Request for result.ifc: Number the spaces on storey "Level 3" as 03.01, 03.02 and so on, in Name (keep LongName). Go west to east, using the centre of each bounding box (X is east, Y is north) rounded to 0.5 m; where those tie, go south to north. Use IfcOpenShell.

First a look at what the model holds.

```python
import ifcopenshell
import ifcopenshell.util.element
import ifcopenshell.util.placement

model = ifcopenshell.open("result.ifc")
print(model.schema)
storey = next(s for s in model.by_type("IfcBuildingStorey") if s.Name == "Level 3")
spaces = [e for e in ifcopenshell.util.element.get_decomposition(storey) if e.is_a("IfcSpace")]
for e in sorted(spaces, key=lambda e: e.id()):
    origin = ifcopenshell.util.placement.get_local_placement(e.ObjectPlacement)[:3, 3]
    print(e.id(), e.Name, e.LongName, origin.round(2) + 0.0, sep=" | ")
```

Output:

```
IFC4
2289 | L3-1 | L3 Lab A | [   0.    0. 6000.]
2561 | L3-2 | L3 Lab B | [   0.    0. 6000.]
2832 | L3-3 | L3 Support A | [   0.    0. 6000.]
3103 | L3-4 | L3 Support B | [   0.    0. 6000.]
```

```python
import ifcopenshell
import ifcopenshell.geom
import ifcopenshell.util.element
import ifcopenshell.util.shape

model = ifcopenshell.open("result.ifc")
settings = ifcopenshell.geom.settings()
settings.set("use-world-coords", True)


def centre(element):
    shape = ifcopenshell.geom.create_shape(settings, element)
    return ifcopenshell.util.shape.get_bbox_centroid(shape.geometry)


storey = next(s for s in model.by_type("IfcBuildingStorey") if s.Name == "Level 3")
spaces = [e for e in ifcopenshell.util.element.get_decomposition(storey) if e.is_a("IfcSpace")]

# Insertion points can sit at a corner or the storey origin, so sort by the geometry (in metres).
centres = {e: centre(e) for e in spaces}
spaces.sort(key=lambda e: (round(centres[e][0] / 0.5), centres[e][1]))

for i, e in enumerate(spaces, start=1):
    number = f"03.{i:02d}"
    e.Name = number
    print(e.id(), number)

model.write("result-out.ifc")
```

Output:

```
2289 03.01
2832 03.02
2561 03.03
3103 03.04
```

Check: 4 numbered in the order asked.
